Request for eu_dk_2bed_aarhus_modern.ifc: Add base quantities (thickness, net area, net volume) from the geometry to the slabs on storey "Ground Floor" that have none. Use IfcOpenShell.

First a look at what the model holds.

```python
import ifcopenshell
import ifcopenshell.util.element
import ifcopenshell.util.unit

model = ifcopenshell.open("eu_dk_2bed_aarhus_modern.ifc")
print(model.schema)
for unit_type in ("LENGTHUNIT", "AREAUNIT", "VOLUMEUNIT"):
    print(unit_type, ifcopenshell.util.unit.calculate_unit_scale(model, unit_type))
storey = next(s for s in model.by_type("IfcBuildingStorey") if s.Name == "Ground Floor")
slabs = [e for e in ifcopenshell.util.element.get_decomposition(storey) if e.is_a("IfcSlab")]
for e in sorted(slabs, key=lambda e: e.id()):
    print(e.id(), e.is_a(), e.Name, list(ifcopenshell.util.element.get_psets(e, qtos_only=True)), sep=" | ")
```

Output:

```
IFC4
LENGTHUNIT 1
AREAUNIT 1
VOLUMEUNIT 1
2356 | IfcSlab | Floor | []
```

```python
import ifcopenshell
import ifcopenshell.api.pset
import ifcopenshell.geom
import ifcopenshell.util.element
import ifcopenshell.util.shape
import ifcopenshell.util.unit

model = ifcopenshell.open("eu_dk_2bed_aarhus_modern.ifc")
unit_scale = ifcopenshell.util.unit.calculate_unit_scale(model)
area_scale = ifcopenshell.util.unit.calculate_unit_scale(model, "AREAUNIT")
volume_scale = ifcopenshell.util.unit.calculate_unit_scale(model, "VOLUMEUNIT")
settings = ifcopenshell.geom.settings()

storey = next(s for s in model.by_type("IfcBuildingStorey") if s.Name == "Ground Floor")
slabs = [e for e in ifcopenshell.util.element.get_decomposition(storey) if e.is_a("IfcSlab")]

for e in sorted(slabs, key=lambda e: e.id()):
    if ifcopenshell.util.element.get_psets(e, qtos_only=True, should_inherit=False):
        continue
    # Geometry comes back in metres, in the element's own axes.
    shape = ifcopenshell.geom.create_shape(settings, e)
    values = {
        "Width": ifcopenshell.util.shape.get_z(shape.geometry) / unit_scale,
        "NetArea": ifcopenshell.util.shape.get_footprint_area(shape.geometry) / area_scale,
        "NetVolume": ifcopenshell.util.shape.get_volume(shape.geometry) / volume_scale,
    }
    qto = ifcopenshell.api.pset.add_qto(model, product=e, name="Qto_SlabBaseQuantities")
    ifcopenshell.api.pset.edit_qto(model, qto=qto, properties=values)
    print(e.id(), {k: round(v, 3) for k, v in values.items()})

model.write("eu_dk_2bed_aarhus_modern_rev.ifc")
```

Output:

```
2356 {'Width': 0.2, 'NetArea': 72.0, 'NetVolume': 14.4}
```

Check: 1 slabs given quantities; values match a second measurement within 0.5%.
